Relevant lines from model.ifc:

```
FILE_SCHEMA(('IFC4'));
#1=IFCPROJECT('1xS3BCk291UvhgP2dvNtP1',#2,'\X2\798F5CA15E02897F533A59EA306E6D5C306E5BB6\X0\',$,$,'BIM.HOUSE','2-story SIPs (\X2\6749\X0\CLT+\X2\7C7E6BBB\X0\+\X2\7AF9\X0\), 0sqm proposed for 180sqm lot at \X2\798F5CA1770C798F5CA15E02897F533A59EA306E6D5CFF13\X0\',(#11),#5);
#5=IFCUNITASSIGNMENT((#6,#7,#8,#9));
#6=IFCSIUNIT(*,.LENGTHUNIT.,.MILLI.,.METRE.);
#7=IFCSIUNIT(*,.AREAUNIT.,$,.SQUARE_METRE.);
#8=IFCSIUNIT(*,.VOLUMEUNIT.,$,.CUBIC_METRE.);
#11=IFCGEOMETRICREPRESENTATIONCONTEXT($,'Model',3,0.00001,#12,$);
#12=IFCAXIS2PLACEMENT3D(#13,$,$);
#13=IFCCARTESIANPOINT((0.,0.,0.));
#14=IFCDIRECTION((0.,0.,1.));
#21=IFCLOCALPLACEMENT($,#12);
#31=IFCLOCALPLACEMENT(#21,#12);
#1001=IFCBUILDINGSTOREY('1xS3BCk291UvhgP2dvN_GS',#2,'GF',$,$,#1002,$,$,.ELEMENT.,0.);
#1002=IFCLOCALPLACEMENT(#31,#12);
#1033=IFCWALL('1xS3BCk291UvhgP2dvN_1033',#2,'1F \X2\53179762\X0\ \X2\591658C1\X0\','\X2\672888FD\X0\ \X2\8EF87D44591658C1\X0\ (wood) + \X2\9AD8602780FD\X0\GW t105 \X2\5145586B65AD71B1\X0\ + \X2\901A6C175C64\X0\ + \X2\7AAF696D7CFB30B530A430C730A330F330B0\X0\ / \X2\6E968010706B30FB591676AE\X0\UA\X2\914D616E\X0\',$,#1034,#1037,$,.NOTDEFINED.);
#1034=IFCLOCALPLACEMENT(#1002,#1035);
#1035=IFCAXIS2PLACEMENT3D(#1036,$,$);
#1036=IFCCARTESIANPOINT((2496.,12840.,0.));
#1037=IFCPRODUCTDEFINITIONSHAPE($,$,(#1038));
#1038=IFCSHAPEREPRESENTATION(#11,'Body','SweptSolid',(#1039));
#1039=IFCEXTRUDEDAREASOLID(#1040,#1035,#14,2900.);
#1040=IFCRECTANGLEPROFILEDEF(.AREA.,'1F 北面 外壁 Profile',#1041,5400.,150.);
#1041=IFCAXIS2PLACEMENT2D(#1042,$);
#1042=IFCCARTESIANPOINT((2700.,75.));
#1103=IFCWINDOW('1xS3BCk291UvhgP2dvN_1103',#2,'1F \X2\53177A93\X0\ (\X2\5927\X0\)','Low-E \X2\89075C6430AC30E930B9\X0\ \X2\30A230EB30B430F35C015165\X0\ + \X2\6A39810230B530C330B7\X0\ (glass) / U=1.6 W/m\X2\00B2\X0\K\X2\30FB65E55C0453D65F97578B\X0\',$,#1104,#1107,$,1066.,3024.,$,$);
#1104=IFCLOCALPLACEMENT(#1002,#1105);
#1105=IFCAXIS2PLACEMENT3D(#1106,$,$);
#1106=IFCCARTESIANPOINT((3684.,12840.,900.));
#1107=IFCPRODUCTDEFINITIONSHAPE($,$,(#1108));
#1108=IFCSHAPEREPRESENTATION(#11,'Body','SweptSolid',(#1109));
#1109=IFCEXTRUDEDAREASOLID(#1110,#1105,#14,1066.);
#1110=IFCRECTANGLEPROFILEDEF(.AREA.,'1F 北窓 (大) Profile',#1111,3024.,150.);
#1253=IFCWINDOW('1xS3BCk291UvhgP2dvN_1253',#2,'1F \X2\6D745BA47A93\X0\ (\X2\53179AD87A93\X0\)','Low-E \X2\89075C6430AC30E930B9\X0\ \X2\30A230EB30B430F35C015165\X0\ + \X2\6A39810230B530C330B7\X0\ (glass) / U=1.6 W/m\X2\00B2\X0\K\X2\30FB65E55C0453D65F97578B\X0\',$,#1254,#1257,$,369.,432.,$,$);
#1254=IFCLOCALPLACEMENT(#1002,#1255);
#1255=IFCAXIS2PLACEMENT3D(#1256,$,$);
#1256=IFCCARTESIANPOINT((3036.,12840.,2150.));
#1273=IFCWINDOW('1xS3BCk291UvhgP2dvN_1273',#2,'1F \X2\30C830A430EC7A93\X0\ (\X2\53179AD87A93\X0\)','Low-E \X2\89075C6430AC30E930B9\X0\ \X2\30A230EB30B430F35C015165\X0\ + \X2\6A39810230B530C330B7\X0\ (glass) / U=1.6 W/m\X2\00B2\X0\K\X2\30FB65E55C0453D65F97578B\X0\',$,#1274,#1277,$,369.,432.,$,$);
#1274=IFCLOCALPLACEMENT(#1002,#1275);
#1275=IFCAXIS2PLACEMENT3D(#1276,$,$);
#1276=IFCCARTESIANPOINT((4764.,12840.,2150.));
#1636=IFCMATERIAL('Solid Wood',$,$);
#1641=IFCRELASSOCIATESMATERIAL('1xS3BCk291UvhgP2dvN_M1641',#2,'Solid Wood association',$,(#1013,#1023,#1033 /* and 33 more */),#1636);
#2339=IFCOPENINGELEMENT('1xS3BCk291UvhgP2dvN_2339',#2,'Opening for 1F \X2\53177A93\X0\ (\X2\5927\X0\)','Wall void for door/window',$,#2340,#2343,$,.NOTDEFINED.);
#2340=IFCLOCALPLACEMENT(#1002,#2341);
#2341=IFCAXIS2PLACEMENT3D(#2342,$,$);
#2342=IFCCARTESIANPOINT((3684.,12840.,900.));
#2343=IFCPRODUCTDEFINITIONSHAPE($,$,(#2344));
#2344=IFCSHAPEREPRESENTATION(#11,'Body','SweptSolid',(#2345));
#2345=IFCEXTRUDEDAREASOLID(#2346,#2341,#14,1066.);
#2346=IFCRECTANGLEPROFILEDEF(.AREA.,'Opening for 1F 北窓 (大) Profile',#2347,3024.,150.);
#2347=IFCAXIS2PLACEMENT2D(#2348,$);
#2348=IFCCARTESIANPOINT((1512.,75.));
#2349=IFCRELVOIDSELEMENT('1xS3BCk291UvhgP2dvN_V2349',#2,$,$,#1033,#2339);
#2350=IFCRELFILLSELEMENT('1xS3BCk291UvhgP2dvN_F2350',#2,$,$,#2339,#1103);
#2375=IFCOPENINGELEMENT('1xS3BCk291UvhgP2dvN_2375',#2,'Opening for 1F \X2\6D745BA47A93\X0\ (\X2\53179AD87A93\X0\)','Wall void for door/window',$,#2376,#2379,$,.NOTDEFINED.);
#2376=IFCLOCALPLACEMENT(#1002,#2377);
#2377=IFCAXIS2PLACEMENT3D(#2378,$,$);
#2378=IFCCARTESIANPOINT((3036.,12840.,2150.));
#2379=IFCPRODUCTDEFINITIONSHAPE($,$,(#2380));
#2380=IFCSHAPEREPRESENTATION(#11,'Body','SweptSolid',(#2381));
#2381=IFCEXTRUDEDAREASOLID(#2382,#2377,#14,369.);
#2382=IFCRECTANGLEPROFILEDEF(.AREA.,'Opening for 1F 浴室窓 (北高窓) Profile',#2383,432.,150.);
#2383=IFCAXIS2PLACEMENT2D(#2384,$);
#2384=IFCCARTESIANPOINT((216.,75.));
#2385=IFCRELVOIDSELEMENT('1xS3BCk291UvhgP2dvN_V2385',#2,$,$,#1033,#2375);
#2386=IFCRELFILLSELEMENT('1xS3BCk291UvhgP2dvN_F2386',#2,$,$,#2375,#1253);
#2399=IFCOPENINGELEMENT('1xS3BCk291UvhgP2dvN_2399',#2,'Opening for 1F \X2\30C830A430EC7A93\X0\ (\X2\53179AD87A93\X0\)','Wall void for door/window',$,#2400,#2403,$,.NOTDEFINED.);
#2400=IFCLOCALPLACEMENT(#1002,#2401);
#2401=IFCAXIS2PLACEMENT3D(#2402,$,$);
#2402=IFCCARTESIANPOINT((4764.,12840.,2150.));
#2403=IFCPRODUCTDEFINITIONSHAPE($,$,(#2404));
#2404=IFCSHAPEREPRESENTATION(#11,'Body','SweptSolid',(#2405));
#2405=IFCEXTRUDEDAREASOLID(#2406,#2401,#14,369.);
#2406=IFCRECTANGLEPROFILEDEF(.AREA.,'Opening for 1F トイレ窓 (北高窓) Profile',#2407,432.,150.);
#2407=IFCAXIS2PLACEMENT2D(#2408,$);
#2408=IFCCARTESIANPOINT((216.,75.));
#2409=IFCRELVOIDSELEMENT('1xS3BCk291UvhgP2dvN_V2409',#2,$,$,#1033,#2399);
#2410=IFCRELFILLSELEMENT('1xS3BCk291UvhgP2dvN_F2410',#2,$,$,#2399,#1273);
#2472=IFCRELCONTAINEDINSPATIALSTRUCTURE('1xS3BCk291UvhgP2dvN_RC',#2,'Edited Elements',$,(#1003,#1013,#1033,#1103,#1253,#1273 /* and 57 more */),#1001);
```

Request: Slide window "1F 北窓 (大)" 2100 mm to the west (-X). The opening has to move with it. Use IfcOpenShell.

```python
import ifcopenshell
import ifcopenshell.api.geometry
import ifcopenshell.util.placement

model = ifcopenshell.open("model.ifc")

window = model.by_guid("1xS3BCk291UvhgP2dvN_1103")
opening = window.FillsVoids[0].RelatingOpeningElement
wall = opening.VoidsElements[0].RelatingBuildingElement

wall_matrix = ifcopenshell.util.placement.get_local_placement(wall.ObjectPlacement)
shift = wall_matrix[:3, 0] * -2100.0
before = ifcopenshell.util.placement.get_local_placement(window.ObjectPlacement)[:3, 3].copy()

# The window is not placed relative to its opening, so move both.
for product in (opening, window):
    matrix = ifcopenshell.util.placement.get_local_placement(product.ObjectPlacement)
    matrix[:3, 3] += shift
    ifcopenshell.api.geometry.edit_object_placement(model, product=product, matrix=matrix, is_si=False)

after = ifcopenshell.util.placement.get_local_placement(window.ObjectPlacement)[:3, 3]
print("window moved by", (after - before).round(3) + 0.0)

model.write("model_v2.ifc")
```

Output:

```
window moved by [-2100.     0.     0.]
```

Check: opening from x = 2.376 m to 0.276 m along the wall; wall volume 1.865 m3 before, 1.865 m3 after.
